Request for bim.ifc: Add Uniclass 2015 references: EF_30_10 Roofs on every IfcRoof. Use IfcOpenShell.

First a look at what the model holds.

```python
import ifcopenshell

model = ifcopenshell.open("bim.ifc")
print(model.schema)
print("classifications:", [c.Name for c in model.by_type("IfcClassification")])
for ifc_class in ("IfcDoor", "IfcRoof", "IfcStair", "IfcWall", "IfcWindow"):
    print(ifc_class, len(model.by_type(ifc_class)))
```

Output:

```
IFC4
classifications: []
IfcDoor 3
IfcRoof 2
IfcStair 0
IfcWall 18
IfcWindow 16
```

```python
import ifcopenshell
import ifcopenshell.api.classification

model = ifcopenshell.open("bim.ifc")

system = ifcopenshell.api.classification.add_classification(model, classification="Uniclass 2015")

codes = {
    "IfcRoof": ("EF_30_10", "Roofs"),
}
for ifc_class, (code, name) in codes.items():
    products = model.by_type(ifc_class)
    ifcopenshell.api.classification.add_reference(
        model, products=products, classification=system, identification=code, name=name
    )
    print(code, len(products))

model.write("bim_edited.ifc")
```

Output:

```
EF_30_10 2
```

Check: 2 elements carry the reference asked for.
